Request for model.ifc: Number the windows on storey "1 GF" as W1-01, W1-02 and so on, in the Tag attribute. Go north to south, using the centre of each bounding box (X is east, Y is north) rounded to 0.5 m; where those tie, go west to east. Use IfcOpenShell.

First a look at what the model holds.

```python
import ifcopenshell
import ifcopenshell.util.element
import ifcopenshell.util.placement

model = ifcopenshell.open("model.ifc")
print(model.schema)
storey = next(s for s in model.by_type("IfcBuildingStorey") if s.Name == "1 GF")
windows = [e for e in ifcopenshell.util.element.get_decomposition(storey) if e.is_a("IfcWindow")]
for e in sorted(windows, key=lambda e: e.id()):
    origin = ifcopenshell.util.placement.get_local_placement(e.ObjectPlacement)[:3, 3]
    print(e.id(), e.Tag, e.Name, origin.round(2) + 0.0, sep=" | ")
```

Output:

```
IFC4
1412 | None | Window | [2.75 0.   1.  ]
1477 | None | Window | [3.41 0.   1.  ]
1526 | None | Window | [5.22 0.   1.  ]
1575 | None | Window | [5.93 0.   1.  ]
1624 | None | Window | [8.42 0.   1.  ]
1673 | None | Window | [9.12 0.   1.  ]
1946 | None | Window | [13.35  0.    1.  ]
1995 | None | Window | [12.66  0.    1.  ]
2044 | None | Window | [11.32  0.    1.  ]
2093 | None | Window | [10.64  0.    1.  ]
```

```python
import ifcopenshell
import ifcopenshell.geom
import ifcopenshell.util.element
import ifcopenshell.util.shape

model = ifcopenshell.open("model.ifc")
settings = ifcopenshell.geom.settings()
settings.set("use-world-coords", True)


def centre(element):
    shape = ifcopenshell.geom.create_shape(settings, element)
    return ifcopenshell.util.shape.get_bbox_centroid(shape.geometry)


storey = next(s for s in model.by_type("IfcBuildingStorey") if s.Name == "1 GF")
windows = [e for e in ifcopenshell.util.element.get_decomposition(storey) if e.is_a("IfcWindow")]

# Insertion points can sit at a corner or the storey origin, so sort by the geometry (in metres).
centres = {e: centre(e) for e in windows}
windows.sort(key=lambda e: (-round(centres[e][1] / 0.5), centres[e][0]))

for i, e in enumerate(windows, start=1):
    number = f"W1-{i:02d}"
    e.Tag = number
    print(e.id(), number)

model.write("model-out.ifc")
```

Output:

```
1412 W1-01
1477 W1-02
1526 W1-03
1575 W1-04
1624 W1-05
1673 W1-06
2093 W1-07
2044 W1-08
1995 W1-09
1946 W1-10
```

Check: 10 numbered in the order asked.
